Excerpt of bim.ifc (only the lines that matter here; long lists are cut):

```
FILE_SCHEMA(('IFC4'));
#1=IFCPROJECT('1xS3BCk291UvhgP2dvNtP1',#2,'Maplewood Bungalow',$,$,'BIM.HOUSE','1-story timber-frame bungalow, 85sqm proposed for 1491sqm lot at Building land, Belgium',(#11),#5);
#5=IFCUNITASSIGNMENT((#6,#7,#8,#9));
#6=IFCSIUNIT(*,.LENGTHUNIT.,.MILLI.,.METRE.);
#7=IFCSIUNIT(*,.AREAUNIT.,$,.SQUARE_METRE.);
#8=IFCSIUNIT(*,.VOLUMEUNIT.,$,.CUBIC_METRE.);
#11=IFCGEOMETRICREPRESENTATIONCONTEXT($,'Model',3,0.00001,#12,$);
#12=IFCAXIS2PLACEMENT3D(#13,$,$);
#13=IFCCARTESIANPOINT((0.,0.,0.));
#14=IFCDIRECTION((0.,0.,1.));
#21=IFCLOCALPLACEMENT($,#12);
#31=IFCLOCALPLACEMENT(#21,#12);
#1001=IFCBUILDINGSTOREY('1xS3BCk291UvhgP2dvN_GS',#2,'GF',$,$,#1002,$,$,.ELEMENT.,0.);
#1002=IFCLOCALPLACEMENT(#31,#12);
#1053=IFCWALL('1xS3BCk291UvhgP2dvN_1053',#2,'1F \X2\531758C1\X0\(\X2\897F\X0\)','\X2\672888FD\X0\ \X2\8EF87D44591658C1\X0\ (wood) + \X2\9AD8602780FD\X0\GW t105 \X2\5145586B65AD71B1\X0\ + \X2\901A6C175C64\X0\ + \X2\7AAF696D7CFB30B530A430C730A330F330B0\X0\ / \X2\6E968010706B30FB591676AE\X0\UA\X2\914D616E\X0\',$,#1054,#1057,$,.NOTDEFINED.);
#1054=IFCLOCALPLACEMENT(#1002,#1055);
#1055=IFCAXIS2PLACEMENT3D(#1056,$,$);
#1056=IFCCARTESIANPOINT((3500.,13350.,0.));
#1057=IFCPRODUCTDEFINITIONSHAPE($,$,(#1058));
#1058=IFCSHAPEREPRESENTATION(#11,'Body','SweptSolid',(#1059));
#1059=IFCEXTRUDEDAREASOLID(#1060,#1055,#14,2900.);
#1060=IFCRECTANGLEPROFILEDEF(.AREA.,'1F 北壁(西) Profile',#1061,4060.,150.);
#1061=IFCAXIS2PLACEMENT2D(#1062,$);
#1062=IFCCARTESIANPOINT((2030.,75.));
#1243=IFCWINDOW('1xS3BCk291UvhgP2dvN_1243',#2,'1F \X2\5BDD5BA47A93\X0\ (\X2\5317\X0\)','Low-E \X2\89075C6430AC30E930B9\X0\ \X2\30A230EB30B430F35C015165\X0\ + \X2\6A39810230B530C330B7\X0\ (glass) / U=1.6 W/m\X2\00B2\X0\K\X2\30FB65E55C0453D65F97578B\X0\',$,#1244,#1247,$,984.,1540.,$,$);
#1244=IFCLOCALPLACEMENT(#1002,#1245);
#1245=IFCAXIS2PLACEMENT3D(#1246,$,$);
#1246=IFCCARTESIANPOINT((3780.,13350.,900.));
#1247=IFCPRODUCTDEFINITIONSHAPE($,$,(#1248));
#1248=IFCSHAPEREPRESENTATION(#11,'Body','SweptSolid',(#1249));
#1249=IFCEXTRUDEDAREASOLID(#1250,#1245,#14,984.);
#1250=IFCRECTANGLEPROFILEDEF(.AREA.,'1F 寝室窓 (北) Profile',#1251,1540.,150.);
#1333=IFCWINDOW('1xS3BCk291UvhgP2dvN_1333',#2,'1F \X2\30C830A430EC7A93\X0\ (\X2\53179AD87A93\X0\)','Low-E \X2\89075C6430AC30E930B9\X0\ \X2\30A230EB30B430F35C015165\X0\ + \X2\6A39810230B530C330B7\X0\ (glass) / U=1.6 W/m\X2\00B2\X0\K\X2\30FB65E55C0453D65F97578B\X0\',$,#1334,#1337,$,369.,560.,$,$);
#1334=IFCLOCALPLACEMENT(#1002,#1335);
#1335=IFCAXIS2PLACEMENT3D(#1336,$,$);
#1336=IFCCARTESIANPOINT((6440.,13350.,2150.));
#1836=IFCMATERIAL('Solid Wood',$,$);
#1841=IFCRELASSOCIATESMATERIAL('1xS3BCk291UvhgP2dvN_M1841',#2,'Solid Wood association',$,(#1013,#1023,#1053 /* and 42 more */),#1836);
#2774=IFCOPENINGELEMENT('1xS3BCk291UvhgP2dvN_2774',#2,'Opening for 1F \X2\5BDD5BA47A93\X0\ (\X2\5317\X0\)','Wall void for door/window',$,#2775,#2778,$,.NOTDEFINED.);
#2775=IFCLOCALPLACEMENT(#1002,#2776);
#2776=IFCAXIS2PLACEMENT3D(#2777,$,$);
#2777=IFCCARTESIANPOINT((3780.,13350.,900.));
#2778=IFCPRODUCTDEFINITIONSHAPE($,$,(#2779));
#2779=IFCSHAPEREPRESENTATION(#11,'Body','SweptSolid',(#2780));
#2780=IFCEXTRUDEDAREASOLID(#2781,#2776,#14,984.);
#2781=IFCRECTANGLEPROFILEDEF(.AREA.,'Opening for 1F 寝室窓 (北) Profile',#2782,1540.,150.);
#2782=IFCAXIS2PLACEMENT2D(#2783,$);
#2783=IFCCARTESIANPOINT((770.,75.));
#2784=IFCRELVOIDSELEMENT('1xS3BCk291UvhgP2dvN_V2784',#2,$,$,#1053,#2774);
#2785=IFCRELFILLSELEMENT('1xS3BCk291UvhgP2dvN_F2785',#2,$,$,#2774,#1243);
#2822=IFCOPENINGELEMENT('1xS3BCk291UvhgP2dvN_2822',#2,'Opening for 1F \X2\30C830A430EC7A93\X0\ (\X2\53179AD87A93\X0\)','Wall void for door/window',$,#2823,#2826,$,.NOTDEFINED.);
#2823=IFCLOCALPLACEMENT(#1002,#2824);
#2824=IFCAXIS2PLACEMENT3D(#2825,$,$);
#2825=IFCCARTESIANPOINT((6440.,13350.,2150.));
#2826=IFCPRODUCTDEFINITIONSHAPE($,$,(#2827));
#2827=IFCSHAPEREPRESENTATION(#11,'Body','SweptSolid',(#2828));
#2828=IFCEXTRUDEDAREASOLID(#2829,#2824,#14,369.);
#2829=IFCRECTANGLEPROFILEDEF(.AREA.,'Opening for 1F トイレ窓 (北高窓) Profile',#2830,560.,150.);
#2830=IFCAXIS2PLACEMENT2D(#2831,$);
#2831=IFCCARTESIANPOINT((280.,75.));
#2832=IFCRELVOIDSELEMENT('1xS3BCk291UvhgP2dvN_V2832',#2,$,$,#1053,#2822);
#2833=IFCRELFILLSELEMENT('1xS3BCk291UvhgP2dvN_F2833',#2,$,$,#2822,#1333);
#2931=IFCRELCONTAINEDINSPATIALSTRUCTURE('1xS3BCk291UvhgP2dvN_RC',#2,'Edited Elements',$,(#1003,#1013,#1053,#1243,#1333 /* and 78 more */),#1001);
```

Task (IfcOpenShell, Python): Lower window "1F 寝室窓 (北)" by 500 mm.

```python
import numpy as np
import ifcopenshell
import ifcopenshell.api.geometry
import ifcopenshell.util.placement
import ifcopenshell.util.unit

model = ifcopenshell.open("bim.ifc")
unit_scale = ifcopenshell.util.unit.calculate_unit_scale(model)

window = model.by_guid("1xS3BCk291UvhgP2dvN_1243")
opening = window.FillsVoids[0].RelatingOpeningElement
dz = -0.5 / unit_scale

shift = np.array([0.0, 0.0, dz])
# The window is not placed relative to its opening, so move both.
for product in (opening, window):
    matrix = ifcopenshell.util.placement.get_local_placement(product.ObjectPlacement)
    matrix[:3, 3] += shift
    ifcopenshell.api.geometry.edit_object_placement(model, product=product, matrix=matrix, is_si=False)

print(f"moved by {dz * unit_scale:+.3f} m")

model.write("bim_rev.ifc")
```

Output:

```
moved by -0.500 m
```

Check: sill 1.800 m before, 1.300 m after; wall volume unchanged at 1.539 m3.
